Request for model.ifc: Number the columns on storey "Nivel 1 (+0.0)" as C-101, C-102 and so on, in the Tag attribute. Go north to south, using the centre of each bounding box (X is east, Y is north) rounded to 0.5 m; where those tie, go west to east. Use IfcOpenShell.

First a look at what the model holds.

```python
import ifcopenshell
import ifcopenshell.util.element
import ifcopenshell.util.placement

model = ifcopenshell.open("model.ifc")
print(model.schema)
storey = next(s for s in model.by_type("IfcBuildingStorey") if s.Name == "Nivel 1 (+0.0)")
columns = [e for e in ifcopenshell.util.element.get_decomposition(storey) if e.is_a("IfcColumn")]
for e in sorted(columns, key=lambda e: e.id()):
    origin = ifcopenshell.util.placement.get_local_placement(e.ObjectPlacement)[:3, 3]
    print(e.id(), e.Tag, e.Name, origin.round(2) + 0.0, sep=" | ")
```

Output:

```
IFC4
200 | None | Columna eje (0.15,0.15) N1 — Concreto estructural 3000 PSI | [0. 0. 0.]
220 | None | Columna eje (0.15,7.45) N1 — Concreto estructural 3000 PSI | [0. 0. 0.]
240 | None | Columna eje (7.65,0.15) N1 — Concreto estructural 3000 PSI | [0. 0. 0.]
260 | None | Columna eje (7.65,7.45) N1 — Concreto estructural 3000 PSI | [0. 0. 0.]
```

```python
import ifcopenshell
import ifcopenshell.geom
import ifcopenshell.util.element
import ifcopenshell.util.shape

model = ifcopenshell.open("model.ifc")
settings = ifcopenshell.geom.settings()
settings.set("use-world-coords", True)


def centre(element):
    shape = ifcopenshell.geom.create_shape(settings, element)
    return ifcopenshell.util.shape.get_bbox_centroid(shape.geometry)


storey = next(s for s in model.by_type("IfcBuildingStorey") if s.Name == "Nivel 1 (+0.0)")
columns = [e for e in ifcopenshell.util.element.get_decomposition(storey) if e.is_a("IfcColumn")]

# Insertion points can sit at a corner or the storey origin, so sort by the geometry (in metres).
centres = {e: centre(e) for e in columns}
columns.sort(key=lambda e: (-round(centres[e][1] / 0.5), centres[e][0]))

for i, e in enumerate(columns, start=1):
    number = f"C-1{i:02d}"
    e.Tag = number
    print(e.id(), number)

model.write("model-out.ifc")
```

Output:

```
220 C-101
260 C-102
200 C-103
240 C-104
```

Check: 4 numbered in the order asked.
